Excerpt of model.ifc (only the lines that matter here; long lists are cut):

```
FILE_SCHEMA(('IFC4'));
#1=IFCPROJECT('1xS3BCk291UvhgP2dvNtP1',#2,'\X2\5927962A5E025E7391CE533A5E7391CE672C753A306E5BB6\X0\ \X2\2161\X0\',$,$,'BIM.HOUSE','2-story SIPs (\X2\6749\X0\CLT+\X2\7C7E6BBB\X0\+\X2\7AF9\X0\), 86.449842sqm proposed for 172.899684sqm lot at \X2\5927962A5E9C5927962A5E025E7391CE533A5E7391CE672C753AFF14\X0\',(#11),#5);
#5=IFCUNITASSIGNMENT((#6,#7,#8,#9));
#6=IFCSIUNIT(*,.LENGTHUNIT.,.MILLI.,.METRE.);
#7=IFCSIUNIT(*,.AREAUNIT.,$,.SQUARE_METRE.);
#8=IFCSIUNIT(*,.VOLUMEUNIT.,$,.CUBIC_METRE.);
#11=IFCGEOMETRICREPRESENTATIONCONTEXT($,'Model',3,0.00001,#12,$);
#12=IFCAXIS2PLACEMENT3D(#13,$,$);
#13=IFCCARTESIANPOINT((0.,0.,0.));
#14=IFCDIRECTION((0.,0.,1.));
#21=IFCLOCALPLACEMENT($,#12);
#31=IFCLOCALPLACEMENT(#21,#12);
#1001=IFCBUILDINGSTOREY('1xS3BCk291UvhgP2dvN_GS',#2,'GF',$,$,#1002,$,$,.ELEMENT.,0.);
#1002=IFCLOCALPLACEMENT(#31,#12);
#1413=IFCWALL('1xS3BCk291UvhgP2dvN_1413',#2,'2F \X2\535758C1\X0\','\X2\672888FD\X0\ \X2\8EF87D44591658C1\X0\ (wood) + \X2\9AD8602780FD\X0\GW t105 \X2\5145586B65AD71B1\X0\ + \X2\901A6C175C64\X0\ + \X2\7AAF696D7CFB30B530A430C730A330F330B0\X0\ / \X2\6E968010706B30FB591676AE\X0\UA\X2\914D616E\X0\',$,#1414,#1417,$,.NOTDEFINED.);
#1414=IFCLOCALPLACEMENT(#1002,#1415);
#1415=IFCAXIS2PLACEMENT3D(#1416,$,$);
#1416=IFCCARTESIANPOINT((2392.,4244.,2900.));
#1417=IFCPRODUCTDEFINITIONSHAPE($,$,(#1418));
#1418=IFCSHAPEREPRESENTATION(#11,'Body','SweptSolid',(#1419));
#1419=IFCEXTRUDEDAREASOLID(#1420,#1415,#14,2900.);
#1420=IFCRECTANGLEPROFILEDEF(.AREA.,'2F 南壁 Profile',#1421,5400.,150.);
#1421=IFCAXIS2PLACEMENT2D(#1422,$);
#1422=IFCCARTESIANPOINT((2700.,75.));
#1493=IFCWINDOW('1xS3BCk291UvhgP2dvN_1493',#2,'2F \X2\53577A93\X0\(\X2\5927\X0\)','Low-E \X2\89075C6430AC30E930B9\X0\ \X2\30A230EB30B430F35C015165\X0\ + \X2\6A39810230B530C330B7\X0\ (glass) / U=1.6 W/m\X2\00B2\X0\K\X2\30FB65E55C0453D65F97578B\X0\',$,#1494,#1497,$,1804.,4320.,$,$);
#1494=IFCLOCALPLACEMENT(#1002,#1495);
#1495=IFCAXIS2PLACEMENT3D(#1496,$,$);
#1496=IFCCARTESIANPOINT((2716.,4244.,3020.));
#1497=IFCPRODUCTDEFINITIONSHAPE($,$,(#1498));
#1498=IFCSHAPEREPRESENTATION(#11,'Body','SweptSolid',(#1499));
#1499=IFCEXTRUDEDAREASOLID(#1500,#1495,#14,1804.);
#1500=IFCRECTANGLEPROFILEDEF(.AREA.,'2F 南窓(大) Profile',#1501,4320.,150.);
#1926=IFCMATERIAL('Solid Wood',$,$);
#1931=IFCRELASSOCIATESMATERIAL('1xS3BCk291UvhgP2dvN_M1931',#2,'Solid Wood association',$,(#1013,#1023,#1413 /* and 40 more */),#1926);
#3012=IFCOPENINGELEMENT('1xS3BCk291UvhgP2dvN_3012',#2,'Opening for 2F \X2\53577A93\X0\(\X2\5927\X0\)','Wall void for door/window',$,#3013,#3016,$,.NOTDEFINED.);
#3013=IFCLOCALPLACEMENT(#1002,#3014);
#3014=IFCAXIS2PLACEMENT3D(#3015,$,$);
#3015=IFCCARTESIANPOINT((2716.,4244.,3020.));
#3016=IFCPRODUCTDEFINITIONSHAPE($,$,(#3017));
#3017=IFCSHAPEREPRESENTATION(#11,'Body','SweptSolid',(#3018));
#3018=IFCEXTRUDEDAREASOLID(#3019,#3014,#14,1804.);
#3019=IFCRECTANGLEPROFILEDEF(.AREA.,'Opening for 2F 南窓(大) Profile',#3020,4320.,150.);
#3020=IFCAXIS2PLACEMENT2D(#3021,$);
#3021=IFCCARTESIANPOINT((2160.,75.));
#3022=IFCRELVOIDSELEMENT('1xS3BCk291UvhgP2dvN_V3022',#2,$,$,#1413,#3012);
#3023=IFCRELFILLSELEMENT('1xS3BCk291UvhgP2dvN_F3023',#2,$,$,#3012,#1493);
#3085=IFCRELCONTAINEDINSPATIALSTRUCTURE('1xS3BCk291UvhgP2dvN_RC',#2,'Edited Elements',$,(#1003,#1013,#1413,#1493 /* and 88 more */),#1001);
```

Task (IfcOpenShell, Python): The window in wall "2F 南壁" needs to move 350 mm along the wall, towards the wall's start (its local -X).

```python
import ifcopenshell
import ifcopenshell.api.geometry
import ifcopenshell.util.placement

model = ifcopenshell.open("model.ifc")

window = model.by_guid("1xS3BCk291UvhgP2dvN_1493")
opening = window.FillsVoids[0].RelatingOpeningElement
wall = opening.VoidsElements[0].RelatingBuildingElement

wall_matrix = ifcopenshell.util.placement.get_local_placement(wall.ObjectPlacement)
shift = wall_matrix[:3, 0] * -350.0
before = ifcopenshell.util.placement.get_local_placement(window.ObjectPlacement)[:3, 3].copy()

# The window is not placed relative to its opening, so move both.
for product in (opening, window):
    matrix = ifcopenshell.util.placement.get_local_placement(product.ObjectPlacement)
    matrix[:3, 3] += shift
    ifcopenshell.api.geometry.edit_object_placement(model, product=product, matrix=matrix, is_si=False)

after = ifcopenshell.util.placement.get_local_placement(window.ObjectPlacement)[:3, 3]
print("window moved by", (after - before).round(3) + 0.0)

model.write("model_rev.ifc")
```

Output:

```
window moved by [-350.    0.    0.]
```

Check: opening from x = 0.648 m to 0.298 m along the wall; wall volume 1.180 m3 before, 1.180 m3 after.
